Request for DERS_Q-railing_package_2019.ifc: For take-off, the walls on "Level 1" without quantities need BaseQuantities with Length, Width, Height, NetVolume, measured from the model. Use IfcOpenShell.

First a look at what the model holds.

```python
import ifcopenshell
import ifcopenshell.util.element
import ifcopenshell.util.unit

model = ifcopenshell.open("DERS_Q-railing_package_2019.ifc")
print(model.schema)
for unit_type in ("LENGTHUNIT", "AREAUNIT", "VOLUMEUNIT"):
    print(unit_type, ifcopenshell.util.unit.calculate_unit_scale(model, unit_type))
storey = next(s for s in model.by_type("IfcBuildingStorey") if s.Name == "Level 1")
walls = [e for e in ifcopenshell.util.element.get_decomposition(storey) if e.is_a("IfcWall")]
for e in sorted(walls, key=lambda e: e.id()):
    print(e.id(), e.is_a(), e.Name, list(ifcopenshell.util.element.get_psets(e, qtos_only=True)), sep=" | ")
```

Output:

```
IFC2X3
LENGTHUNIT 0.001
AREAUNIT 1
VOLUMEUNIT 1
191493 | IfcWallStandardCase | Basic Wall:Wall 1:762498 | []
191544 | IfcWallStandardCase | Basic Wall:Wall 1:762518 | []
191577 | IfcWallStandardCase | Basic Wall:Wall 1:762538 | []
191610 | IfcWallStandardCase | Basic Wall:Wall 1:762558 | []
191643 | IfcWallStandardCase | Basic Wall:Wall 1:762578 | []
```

```python
import ifcopenshell
import ifcopenshell.api.pset
import ifcopenshell.geom
import ifcopenshell.util.element
import ifcopenshell.util.shape
import ifcopenshell.util.unit

model = ifcopenshell.open("DERS_Q-railing_package_2019.ifc")
unit_scale = ifcopenshell.util.unit.calculate_unit_scale(model)
volume_scale = ifcopenshell.util.unit.calculate_unit_scale(model, "VOLUMEUNIT")
settings = ifcopenshell.geom.settings()

storey = next(s for s in model.by_type("IfcBuildingStorey") if s.Name == "Level 1")
walls = [e for e in ifcopenshell.util.element.get_decomposition(storey) if e.is_a("IfcWall")]

for e in sorted(walls, key=lambda e: e.id()):
    if ifcopenshell.util.element.get_psets(e, qtos_only=True, should_inherit=False):
        continue
    # Geometry comes back in metres, in the element's own axes.
    shape = ifcopenshell.geom.create_shape(settings, e)
    values = {
        "Length": ifcopenshell.util.shape.get_x(shape.geometry) / unit_scale,
        "Width": ifcopenshell.util.shape.get_y(shape.geometry) / unit_scale,
        "Height": ifcopenshell.util.shape.get_z(shape.geometry) / unit_scale,
        "NetVolume": ifcopenshell.util.shape.get_volume(shape.geometry) / volume_scale,
    }
    qto = ifcopenshell.api.pset.add_qto(model, product=e, name="BaseQuantities")
    ifcopenshell.api.pset.edit_qto(model, qto=qto, properties=values)
    print(e.id(), {k: round(v, 3) for k, v in values.items()})

model.write("DERS_Q-railing_package_2019_v2.ifc")
```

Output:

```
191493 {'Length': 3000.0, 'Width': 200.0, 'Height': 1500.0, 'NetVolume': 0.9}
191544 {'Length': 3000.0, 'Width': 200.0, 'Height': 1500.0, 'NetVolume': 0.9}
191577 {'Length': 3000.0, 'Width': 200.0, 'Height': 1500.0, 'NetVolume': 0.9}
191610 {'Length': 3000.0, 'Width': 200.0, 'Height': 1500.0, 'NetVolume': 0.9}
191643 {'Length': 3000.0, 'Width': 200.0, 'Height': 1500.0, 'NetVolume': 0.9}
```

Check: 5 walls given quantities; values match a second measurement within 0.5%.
